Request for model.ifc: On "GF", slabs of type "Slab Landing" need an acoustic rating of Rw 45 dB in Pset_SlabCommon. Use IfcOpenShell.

First a look at what the model holds.

```python
import ifcopenshell
import ifcopenshell.util.element

model = ifcopenshell.open("model.ifc")
print(model.schema)
storey = next(s for s in model.by_type("IfcBuildingStorey") if s.Name == "GF")
slabs = [e for e in ifcopenshell.util.element.get_decomposition(storey) if e.is_a("IfcSlab")]
seen = {}
for e in slabs:
    element_type = ifcopenshell.util.element.get_type(e)
    key = (element_type.Name if element_type != e and element_type else None, ifcopenshell.util.element.get_pset(e, "Pset_SlabCommon", "AcousticRating"))
    seen[key] = seen.get(key, 0) + 1
for (name, value), count in sorted(seen.items(), key=str):
    print(count, "x", name, "|", value)
```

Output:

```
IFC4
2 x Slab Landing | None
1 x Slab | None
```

```python
import ifcopenshell
import ifcopenshell.api.pset
import ifcopenshell.util.element

model = ifcopenshell.open("model.ifc")

storey = next(s for s in model.by_type("IfcBuildingStorey") if s.Name == "GF")
slabs = [e for e in ifcopenshell.util.element.get_decomposition(storey) if e.is_a("IfcSlab")]

count = 0
for e in slabs:
    element_type = ifcopenshell.util.element.get_type(e)
    if element_type in (None, e) or element_type.Name != "Slab Landing":
        continue
    # add_pset returns the element's existing set when there is one.
    pset = ifcopenshell.api.pset.add_pset(model, product=e, name="Pset_SlabCommon")
    ifcopenshell.api.pset.edit_pset(model, pset=pset, properties={"AcousticRating": "Rw 45 dB"})
    count += 1

print(count, "slabs updated")

model.write("model_edited.ifc")
```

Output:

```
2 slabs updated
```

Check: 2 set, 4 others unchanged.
